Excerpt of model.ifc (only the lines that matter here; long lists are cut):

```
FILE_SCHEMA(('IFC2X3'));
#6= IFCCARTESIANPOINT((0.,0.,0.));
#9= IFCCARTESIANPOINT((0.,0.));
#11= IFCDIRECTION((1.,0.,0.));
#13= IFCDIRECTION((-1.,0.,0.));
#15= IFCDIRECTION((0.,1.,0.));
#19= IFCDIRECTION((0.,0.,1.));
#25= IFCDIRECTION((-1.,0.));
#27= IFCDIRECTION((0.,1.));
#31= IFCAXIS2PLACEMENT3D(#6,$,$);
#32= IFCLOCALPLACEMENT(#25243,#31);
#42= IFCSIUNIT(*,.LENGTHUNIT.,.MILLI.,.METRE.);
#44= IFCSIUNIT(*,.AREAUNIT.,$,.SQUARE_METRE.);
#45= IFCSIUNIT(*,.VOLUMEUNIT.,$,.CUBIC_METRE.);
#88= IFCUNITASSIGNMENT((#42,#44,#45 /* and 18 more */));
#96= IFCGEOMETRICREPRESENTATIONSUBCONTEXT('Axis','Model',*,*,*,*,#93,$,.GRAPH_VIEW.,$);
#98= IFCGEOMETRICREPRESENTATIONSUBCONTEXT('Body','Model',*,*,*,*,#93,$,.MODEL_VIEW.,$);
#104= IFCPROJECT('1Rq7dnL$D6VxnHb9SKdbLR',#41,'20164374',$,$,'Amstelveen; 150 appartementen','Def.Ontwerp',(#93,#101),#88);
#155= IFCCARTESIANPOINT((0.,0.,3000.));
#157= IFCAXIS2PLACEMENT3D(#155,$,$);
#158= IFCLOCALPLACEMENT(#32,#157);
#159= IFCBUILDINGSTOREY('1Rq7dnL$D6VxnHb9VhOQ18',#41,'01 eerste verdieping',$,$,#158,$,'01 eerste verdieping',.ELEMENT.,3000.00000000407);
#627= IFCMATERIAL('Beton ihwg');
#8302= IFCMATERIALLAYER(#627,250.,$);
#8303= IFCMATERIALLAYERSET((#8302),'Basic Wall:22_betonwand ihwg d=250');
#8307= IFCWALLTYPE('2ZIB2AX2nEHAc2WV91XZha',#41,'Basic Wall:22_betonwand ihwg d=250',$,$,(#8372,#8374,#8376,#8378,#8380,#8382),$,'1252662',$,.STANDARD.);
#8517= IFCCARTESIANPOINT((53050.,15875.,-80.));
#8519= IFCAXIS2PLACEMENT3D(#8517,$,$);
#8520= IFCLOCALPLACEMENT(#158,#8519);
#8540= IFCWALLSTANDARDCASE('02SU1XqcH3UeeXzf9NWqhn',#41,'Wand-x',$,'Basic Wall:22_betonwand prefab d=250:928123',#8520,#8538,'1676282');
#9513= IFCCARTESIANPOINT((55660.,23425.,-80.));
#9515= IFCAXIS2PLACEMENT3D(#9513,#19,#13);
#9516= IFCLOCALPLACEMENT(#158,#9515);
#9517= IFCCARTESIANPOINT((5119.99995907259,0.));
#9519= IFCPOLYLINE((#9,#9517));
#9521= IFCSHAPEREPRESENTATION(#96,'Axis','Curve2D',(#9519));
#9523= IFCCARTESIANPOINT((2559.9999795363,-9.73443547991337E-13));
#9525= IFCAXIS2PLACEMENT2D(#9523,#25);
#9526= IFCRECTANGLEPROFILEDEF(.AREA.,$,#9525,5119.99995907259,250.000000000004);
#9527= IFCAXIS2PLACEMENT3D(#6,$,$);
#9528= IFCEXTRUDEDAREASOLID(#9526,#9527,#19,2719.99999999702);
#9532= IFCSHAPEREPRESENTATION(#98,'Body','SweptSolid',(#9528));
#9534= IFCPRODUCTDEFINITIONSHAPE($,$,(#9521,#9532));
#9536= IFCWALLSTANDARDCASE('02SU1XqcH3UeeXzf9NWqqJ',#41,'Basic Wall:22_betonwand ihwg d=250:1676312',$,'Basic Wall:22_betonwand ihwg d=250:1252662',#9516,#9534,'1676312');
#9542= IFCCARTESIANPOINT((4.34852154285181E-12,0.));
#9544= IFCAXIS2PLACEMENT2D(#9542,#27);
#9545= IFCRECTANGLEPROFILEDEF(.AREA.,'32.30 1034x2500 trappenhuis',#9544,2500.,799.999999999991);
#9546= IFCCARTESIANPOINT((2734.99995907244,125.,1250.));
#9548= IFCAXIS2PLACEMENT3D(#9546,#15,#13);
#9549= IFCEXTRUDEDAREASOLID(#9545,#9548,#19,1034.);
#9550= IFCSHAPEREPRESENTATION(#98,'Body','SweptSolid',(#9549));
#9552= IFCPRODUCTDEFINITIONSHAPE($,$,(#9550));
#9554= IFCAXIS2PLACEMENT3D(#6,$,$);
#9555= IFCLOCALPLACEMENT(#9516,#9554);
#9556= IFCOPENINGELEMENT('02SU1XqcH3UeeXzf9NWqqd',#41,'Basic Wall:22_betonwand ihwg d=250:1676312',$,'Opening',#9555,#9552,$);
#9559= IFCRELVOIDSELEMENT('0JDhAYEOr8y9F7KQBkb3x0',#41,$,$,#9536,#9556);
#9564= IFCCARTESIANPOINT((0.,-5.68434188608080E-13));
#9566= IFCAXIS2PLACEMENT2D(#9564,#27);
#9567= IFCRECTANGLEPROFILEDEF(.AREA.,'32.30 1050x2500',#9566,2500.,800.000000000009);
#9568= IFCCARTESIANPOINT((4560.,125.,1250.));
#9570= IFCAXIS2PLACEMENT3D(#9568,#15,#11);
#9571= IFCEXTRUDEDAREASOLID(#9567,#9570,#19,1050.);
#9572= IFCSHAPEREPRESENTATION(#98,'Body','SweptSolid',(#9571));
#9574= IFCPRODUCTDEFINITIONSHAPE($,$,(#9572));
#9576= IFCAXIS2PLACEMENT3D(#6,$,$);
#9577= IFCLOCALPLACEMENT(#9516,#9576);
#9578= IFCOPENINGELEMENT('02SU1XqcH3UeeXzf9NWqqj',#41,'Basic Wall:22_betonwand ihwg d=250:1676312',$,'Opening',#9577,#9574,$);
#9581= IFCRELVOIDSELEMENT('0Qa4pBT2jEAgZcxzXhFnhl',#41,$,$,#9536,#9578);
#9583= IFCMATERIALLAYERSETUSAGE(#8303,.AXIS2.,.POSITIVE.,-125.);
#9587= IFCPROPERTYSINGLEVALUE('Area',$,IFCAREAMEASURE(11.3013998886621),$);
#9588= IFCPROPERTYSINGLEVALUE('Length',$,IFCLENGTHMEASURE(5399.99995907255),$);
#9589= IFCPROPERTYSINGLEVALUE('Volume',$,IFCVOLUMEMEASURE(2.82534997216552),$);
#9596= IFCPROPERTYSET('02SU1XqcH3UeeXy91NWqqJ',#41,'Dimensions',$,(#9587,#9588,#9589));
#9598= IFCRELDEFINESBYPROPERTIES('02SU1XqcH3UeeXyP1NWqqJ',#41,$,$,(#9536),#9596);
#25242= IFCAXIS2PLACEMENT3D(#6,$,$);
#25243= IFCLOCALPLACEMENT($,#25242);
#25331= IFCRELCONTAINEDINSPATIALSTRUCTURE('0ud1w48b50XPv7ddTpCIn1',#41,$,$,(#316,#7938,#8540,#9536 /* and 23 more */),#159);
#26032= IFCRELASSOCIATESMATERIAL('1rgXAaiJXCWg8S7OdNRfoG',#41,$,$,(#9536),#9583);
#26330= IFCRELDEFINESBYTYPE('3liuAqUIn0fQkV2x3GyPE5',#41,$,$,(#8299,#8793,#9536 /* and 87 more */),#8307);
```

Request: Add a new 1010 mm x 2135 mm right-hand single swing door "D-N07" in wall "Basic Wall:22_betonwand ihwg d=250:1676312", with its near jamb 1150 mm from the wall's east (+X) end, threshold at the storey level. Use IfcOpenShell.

```python
import numpy as np
import ifcopenshell
import ifcopenshell.api.feature
import ifcopenshell.api.geometry
import ifcopenshell.api.pset
import ifcopenshell.api.root
import ifcopenshell.api.spatial
import ifcopenshell.api.type
import ifcopenshell.geom
import ifcopenshell.util.element
import ifcopenshell.util.placement
import ifcopenshell.util.representation
import ifcopenshell.util.shape
import ifcopenshell.util.unit

model = ifcopenshell.open("model.ifc")
unit_scale = ifcopenshell.util.unit.calculate_unit_scale(model)
area_scale = ifcopenshell.util.unit.calculate_unit_scale(model, "AREAUNIT")
volume_scale = ifcopenshell.util.unit.calculate_unit_scale(model, "VOLUMEUNIT")
settings = ifcopenshell.geom.settings()


def volume(element):
    """Net volume in cubic metres, openings subtracted."""
    shape = ifcopenshell.geom.create_shape(settings, element)
    return ifcopenshell.util.shape.get_volume(shape.geometry)


wall = model.by_guid("02SU1XqcH3UeeXzf9NWqqJ")
storey = ifcopenshell.util.element.get_container(wall, ifc_class="IfcBuildingStorey")
context = ifcopenshell.util.representation.get_context(model, "Model", "Body", "MODEL_VIEW")
before = volume(wall)

width, height, from_end, sill = 1.01, 2.135, 1.15, 0.0  # metres

# The wall runs along its own X axis, and the end named is its -X end.
wall_shape = ifcopenshell.geom.create_shape(settings, wall)
x, y, z = ifcopenshell.util.shape.get_vertices(wall_shape.geometry).T
start = x.min() + from_end
face, thickness = float(y.min()), float(y.max() - y.min())
wall_matrix = ifcopenshell.util.placement.get_local_placement(wall.ObjectPlacement)
level = ifcopenshell.util.placement.get_local_placement(storey.ObjectPlacement)[2, 3]


def in_wall(x, y):
    """Placement at x, y metres in the wall's axes, at sill height."""
    matrix = wall_matrix.copy()
    matrix[:, 3] = wall_matrix @ np.array([x / unit_scale, y / unit_scale, 0.0, 1.0])
    matrix[2, 3] = level + sill / unit_scale
    return matrix


# Opening: a box that overshoots both wall faces by 50 mm.
opening = ifcopenshell.api.root.create_entity(model, ifc_class="IfcOpeningElement")
box = ifcopenshell.api.geometry.add_wall_representation(
    model, context=context, length=width, height=height, thickness=thickness + 0.1
)
ifcopenshell.api.geometry.assign_representation(model, product=opening, representation=box)
ifcopenshell.api.geometry.edit_object_placement(model, product=opening, matrix=in_wall(start, face - 0.05), is_si=False)
ifcopenshell.api.feature.add_feature(model, feature=opening, element=wall)

door = ifcopenshell.api.root.create_entity(model, ifc_class="IfcDoor", name="D-N07")
door.OverallWidth, door.OverallHeight = width / unit_scale, height / unit_scale
body = ifcopenshell.api.geometry.add_door_representation(
    model,
    context=context,
    overall_width=door.OverallWidth,
    overall_height=door.OverallHeight,
    operation_type="SINGLE_SWING_RIGHT",
    lining_properties={"LiningDepth": thickness / unit_scale, "ThresholdDepth": thickness / unit_scale},
)
ifcopenshell.api.geometry.assign_representation(model, product=door, representation=body)
ifcopenshell.api.spatial.assign_container(model, products=[door], relating_structure=storey)
fills = ifcopenshell.api.feature.add_filling(model, opening=opening, element=door)
fills.OwnerHistory = door.OwnerHistory  # required in IFC2X3

# IFC2X3 keeps the operation on the door style.
style = ifcopenshell.api.root.create_entity(model, ifc_class="IfcDoorStyle", name="D-N07")
style.OperationType, style.ConstructionType = "SINGLE_SWING_RIGHT", "NOTDEFINED"
style.ParameterTakesPrecedence = style.Sizeable = False
ifcopenshell.api.type.assign_type(model, related_objects=[door], relating_type=style)

# The lining spans the wall, so the door starts at the wall face.
ifcopenshell.api.geometry.edit_object_placement(model, product=door, matrix=in_wall(start, face), is_si=False)

after = volume(wall)

# Update the wall's stored quantities.
pset = model.by_id(ifcopenshell.util.element.get_pset(wall, "Dimensions", should_inherit=False)["id"])
ifcopenshell.api.pset.edit_pset(model, pset=pset, properties={
    "Area": model.create_entity("IfcAreaMeasure", after / thickness / area_scale),
    "Volume": model.create_entity("IfcVolumeMeasure", after / volume_scale),
})

print(f"wall volume {before:.3f} -> {after:.3f} m3")

model.write("model_updated.ifc")
```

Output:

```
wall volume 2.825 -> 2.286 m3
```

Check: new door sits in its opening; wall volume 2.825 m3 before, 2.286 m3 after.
